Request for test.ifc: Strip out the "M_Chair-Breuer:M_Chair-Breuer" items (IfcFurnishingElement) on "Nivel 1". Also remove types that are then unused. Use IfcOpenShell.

First a look at what the model holds.

```python
import ifcopenshell
import ifcopenshell.util.element

model = ifcopenshell.open("test.ifc")
print(model.schema)
storey = next(s for s in model.by_type("IfcBuildingStorey") if s.Name == "Nivel 1")
furniture = [e for e in ifcopenshell.util.element.get_decomposition(storey) if e.is_a("IfcFurnishingElement")]
seen = {}
for e in furniture:
    element_type = ifcopenshell.util.element.get_type(e)
    name = element_type.Name if element_type not in (None, e) else None
    seen[name] = seen.get(name, 0) + 1
for name, count in sorted(seen.items(), key=str):
    print(count, "x", name)
```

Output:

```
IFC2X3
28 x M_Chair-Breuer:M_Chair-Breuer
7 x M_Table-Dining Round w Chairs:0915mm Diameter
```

```python
import ifcopenshell
import ifcopenshell.api.root
import ifcopenshell.util.element

model = ifcopenshell.open("test.ifc")

storey = next(s for s in model.by_type("IfcBuildingStorey") if s.Name == "Nivel 1")
furniture = [e for e in ifcopenshell.util.element.get_decomposition(storey) if e.is_a("IfcFurnishingElement")]
targets = [e for e in furniture if (t := ifcopenshell.util.element.get_type(e)) not in (None, e) and t.Name == "M_Chair-Breuer:M_Chair-Breuer"]
types = {ifcopenshell.util.element.get_type(e) for e in targets} - {None, *targets}

for e in targets:
    ifcopenshell.api.root.remove_product(model, product=e)
print(len(targets), "removed")

unused = [t for t in types if not ifcopenshell.util.element.get_types(t)]
for t in unused:
    ifcopenshell.api.root.remove_product(model, product=t)
print(len(unused), "unused types removed")

model.write("test_updated.ifc")
```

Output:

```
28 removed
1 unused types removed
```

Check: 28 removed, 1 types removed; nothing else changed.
